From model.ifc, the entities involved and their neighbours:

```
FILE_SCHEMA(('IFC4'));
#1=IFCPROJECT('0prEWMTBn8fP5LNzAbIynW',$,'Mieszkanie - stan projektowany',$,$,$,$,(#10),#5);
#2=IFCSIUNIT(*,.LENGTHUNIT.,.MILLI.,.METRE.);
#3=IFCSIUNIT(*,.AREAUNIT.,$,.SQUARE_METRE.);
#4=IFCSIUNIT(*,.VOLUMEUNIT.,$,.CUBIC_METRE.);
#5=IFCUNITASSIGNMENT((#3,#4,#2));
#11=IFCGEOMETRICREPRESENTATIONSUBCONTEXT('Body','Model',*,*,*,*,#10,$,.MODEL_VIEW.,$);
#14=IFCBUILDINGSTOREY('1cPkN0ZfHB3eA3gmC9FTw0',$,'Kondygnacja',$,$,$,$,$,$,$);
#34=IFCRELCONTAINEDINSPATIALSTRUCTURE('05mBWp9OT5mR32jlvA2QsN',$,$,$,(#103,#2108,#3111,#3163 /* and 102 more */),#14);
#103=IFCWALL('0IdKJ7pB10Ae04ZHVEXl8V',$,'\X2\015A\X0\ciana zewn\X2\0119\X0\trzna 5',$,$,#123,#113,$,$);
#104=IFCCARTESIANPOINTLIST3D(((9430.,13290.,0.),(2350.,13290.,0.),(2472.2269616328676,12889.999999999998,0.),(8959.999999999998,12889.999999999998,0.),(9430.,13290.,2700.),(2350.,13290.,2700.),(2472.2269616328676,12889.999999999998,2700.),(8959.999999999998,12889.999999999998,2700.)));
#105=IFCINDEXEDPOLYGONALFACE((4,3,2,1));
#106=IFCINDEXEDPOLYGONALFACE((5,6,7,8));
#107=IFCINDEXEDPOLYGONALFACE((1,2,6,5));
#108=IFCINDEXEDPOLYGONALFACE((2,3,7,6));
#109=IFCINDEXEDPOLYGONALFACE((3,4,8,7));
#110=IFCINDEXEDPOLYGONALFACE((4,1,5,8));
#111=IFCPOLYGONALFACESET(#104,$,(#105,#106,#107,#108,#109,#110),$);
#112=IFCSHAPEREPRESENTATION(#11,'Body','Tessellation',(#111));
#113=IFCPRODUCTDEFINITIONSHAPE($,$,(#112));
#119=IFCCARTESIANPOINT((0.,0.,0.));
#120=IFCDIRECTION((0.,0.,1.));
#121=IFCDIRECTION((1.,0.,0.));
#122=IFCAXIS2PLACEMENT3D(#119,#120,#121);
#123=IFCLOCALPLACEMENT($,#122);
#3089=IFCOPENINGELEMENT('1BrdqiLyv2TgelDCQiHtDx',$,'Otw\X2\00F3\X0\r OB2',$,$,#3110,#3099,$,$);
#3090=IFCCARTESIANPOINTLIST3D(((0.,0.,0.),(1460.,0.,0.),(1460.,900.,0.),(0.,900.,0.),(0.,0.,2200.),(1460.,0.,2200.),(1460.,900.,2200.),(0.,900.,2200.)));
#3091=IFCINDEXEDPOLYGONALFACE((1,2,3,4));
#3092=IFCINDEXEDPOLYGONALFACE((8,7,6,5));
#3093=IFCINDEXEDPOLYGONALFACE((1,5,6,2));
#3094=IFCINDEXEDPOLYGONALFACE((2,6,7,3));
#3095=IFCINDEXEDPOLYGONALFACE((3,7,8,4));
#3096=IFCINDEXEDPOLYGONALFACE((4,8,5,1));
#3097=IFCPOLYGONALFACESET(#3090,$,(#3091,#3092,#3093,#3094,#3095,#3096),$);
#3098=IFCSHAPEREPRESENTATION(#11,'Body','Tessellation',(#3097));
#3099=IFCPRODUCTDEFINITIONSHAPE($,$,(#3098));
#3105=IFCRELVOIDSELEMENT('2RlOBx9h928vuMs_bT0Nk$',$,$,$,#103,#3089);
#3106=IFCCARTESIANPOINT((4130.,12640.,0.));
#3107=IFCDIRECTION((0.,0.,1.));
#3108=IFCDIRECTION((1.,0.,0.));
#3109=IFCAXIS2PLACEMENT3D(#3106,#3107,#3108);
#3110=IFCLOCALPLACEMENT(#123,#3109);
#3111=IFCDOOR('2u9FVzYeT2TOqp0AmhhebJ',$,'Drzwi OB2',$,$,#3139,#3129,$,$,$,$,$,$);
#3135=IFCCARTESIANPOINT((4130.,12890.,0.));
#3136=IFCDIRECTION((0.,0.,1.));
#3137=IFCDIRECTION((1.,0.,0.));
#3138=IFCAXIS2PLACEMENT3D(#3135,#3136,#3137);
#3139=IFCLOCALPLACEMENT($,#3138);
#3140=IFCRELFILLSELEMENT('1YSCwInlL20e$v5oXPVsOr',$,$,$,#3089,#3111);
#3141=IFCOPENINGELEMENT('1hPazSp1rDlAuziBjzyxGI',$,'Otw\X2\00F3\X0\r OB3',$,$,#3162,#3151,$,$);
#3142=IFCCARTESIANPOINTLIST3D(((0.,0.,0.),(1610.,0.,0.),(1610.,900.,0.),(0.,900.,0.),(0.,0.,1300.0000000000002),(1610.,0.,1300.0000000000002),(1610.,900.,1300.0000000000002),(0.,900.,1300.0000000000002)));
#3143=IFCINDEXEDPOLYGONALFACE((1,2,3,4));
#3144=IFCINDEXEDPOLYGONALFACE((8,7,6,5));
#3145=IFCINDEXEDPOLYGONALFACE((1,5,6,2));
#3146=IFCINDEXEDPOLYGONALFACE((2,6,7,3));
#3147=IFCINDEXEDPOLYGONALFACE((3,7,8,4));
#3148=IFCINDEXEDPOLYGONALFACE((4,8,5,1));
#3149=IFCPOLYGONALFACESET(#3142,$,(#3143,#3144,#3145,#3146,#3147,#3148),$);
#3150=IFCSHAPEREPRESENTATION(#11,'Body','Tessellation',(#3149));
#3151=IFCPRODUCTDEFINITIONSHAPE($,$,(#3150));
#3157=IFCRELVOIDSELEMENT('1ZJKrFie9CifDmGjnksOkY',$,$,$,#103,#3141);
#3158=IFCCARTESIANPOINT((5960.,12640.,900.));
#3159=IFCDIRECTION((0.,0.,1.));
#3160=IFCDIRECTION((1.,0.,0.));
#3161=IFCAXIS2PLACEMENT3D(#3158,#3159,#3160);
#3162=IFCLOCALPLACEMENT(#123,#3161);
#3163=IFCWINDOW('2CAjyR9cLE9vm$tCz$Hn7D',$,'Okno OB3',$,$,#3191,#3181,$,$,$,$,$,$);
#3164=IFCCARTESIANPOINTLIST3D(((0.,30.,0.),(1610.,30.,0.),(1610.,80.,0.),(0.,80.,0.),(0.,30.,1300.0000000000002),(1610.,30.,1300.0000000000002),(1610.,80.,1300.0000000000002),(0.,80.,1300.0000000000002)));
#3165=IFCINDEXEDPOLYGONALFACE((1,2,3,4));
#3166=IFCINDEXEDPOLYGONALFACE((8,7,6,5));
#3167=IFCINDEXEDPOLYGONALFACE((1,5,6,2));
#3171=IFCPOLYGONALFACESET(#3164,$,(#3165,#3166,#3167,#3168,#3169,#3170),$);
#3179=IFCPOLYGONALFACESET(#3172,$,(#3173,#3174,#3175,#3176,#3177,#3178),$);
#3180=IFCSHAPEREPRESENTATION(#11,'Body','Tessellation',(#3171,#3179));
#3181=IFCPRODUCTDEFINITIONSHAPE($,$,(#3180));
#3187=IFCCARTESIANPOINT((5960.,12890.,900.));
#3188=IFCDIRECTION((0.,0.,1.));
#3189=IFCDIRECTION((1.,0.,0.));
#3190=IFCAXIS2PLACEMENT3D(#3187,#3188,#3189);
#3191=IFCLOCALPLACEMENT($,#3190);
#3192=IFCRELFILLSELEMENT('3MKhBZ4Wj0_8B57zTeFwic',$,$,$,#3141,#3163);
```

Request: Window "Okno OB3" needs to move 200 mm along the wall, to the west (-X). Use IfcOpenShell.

```python
import ifcopenshell
import ifcopenshell.api.geometry
import ifcopenshell.util.placement

model = ifcopenshell.open("model.ifc")

window = model.by_guid("2CAjyR9cLE9vm$tCz$Hn7D")
opening = window.FillsVoids[0].RelatingOpeningElement
wall = opening.VoidsElements[0].RelatingBuildingElement

wall_matrix = ifcopenshell.util.placement.get_local_placement(wall.ObjectPlacement)
shift = wall_matrix[:3, 0] * -200.0
before = ifcopenshell.util.placement.get_local_placement(window.ObjectPlacement)[:3, 3].copy()

# The window is not placed relative to its opening, so move both.
for product in (opening, window):
    matrix = ifcopenshell.util.placement.get_local_placement(product.ObjectPlacement)
    matrix[:3, 3] += shift
    ifcopenshell.api.geometry.edit_object_placement(model, product=product, matrix=matrix, is_si=False)

after = ifcopenshell.util.placement.get_local_placement(window.ObjectPlacement)[:3, 3]
print("window moved by", (after - before).round(3) + 0.0)

model.write("model_rev.ifc")
```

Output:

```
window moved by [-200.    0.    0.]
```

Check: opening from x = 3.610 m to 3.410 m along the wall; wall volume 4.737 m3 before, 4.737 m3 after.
